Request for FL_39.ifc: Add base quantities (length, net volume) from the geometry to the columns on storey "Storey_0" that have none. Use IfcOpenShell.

First a look at what the model holds.

```python
import ifcopenshell
import ifcopenshell.util.element
import ifcopenshell.util.unit

model = ifcopenshell.open("FL_39.ifc")
print(model.schema)
for unit_type in ("LENGTHUNIT", "AREAUNIT", "VOLUMEUNIT"):
    print(unit_type, ifcopenshell.util.unit.calculate_unit_scale(model, unit_type))
storey = next(s for s in model.by_type("IfcBuildingStorey") if s.Name == "Storey_0")
columns = [e for e in ifcopenshell.util.element.get_decomposition(storey) if e.is_a("IfcColumn")]
for e in sorted(columns, key=lambda e: e.id()):
    print(e.id(), e.is_a(), e.Name, list(ifcopenshell.util.element.get_psets(e, qtos_only=True)), sep=" | ")
```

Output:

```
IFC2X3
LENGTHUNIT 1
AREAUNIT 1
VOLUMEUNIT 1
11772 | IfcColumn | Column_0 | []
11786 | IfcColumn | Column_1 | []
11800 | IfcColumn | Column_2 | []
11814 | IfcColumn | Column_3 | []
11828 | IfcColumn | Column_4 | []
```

```python
import ifcopenshell
import ifcopenshell.api.pset
import ifcopenshell.geom
import ifcopenshell.util.element
import ifcopenshell.util.shape
import ifcopenshell.util.unit

model = ifcopenshell.open("FL_39.ifc")
unit_scale = ifcopenshell.util.unit.calculate_unit_scale(model)
volume_scale = ifcopenshell.util.unit.calculate_unit_scale(model, "VOLUMEUNIT")
settings = ifcopenshell.geom.settings()

storey = next(s for s in model.by_type("IfcBuildingStorey") if s.Name == "Storey_0")
columns = [e for e in ifcopenshell.util.element.get_decomposition(storey) if e.is_a("IfcColumn")]

for e in sorted(columns, key=lambda e: e.id()):
    if ifcopenshell.util.element.get_psets(e, qtos_only=True, should_inherit=False):
        continue
    # Geometry comes back in metres, in the element's own axes.
    shape = ifcopenshell.geom.create_shape(settings, e)
    values = {
        "Length": ifcopenshell.util.shape.get_z(shape.geometry) / unit_scale,
        "NetVolume": ifcopenshell.util.shape.get_volume(shape.geometry) / volume_scale,
    }
    qto = ifcopenshell.api.pset.add_qto(model, product=e, name="BaseQuantities")
    ifcopenshell.api.pset.edit_qto(model, qto=qto, properties=values)
    print(e.id(), {k: round(v, 3) for k, v in values.items()})

model.write("FL_39_v2.ifc")
```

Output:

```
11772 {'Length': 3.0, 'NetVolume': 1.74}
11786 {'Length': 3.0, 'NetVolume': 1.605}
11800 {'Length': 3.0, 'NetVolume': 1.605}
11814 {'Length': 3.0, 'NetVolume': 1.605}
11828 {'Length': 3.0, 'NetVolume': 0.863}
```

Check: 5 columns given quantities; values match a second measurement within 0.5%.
